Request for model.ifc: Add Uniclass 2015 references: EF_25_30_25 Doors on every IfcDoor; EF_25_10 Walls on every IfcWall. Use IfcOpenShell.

First a look at what the model holds.

```python
import ifcopenshell

model = ifcopenshell.open("model.ifc")
print(model.schema)
print("classifications:", [c.Name for c in model.by_type("IfcClassification")])
for ifc_class in ("IfcDoor", "IfcRoof", "IfcStair", "IfcWall", "IfcWindow"):
    print(ifc_class, len(model.by_type(ifc_class)))
```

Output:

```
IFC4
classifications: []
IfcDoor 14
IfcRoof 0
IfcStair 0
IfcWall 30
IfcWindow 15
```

```python
import ifcopenshell
import ifcopenshell.api.classification

model = ifcopenshell.open("model.ifc")

system = ifcopenshell.api.classification.add_classification(model, classification="Uniclass 2015")

codes = {
    "IfcDoor": ("EF_25_30_25", "Doors"),
    "IfcWall": ("EF_25_10", "Walls"),
}
for ifc_class, (code, name) in codes.items():
    products = model.by_type(ifc_class)
    ifcopenshell.api.classification.add_reference(
        model, products=products, classification=system, identification=code, name=name
    )
    print(code, len(products))

model.write("model_v2.ifc")
```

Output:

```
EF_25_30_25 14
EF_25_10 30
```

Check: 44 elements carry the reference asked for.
